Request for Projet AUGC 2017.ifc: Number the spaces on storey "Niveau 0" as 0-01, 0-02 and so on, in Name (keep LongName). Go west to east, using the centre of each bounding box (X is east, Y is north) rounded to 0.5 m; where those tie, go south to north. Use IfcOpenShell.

First a look at what the model holds.

```python
import ifcopenshell
import ifcopenshell.util.element
import ifcopenshell.util.placement

model = ifcopenshell.open("Projet AUGC 2017.ifc")
print(model.schema)
storey = next(s for s in model.by_type("IfcBuildingStorey") if s.Name == "Niveau 0")
spaces = [e for e in ifcopenshell.util.element.get_decomposition(storey) if e.is_a("IfcSpace")]
for e in sorted(spaces, key=lambda e: e.id()):
    origin = ifcopenshell.util.placement.get_local_placement(e.ObjectPlacement)[:3, 3]
    print(e.id(), e.Name, e.LongName, origin.round(2) + 0.0, sep=" | ")
```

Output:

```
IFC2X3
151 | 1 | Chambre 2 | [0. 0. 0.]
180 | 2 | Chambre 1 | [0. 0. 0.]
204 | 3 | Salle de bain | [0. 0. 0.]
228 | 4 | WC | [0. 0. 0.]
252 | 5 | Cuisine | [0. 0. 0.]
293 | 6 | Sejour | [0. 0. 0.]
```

```python
import ifcopenshell
import ifcopenshell.geom
import ifcopenshell.util.element
import ifcopenshell.util.shape

model = ifcopenshell.open("Projet AUGC 2017.ifc")
settings = ifcopenshell.geom.settings()
settings.set("use-world-coords", True)


def centre(element):
    shape = ifcopenshell.geom.create_shape(settings, element)
    return ifcopenshell.util.shape.get_bbox_centroid(shape.geometry)


storey = next(s for s in model.by_type("IfcBuildingStorey") if s.Name == "Niveau 0")
spaces = [e for e in ifcopenshell.util.element.get_decomposition(storey) if e.is_a("IfcSpace")]

# Insertion points can sit at a corner or the storey origin, so sort by the geometry (in metres).
centres = {e: centre(e) for e in spaces}
spaces.sort(key=lambda e: (round(centres[e][0] / 0.5), centres[e][1]))

for i, e in enumerate(spaces, start=1):
    number = f"0-{i:02d}"
    e.Name = number
    print(e.id(), number)

model.write("Projet AUGC 2017_edited.ifc")
```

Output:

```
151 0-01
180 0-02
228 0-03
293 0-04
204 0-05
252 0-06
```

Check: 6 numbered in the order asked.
